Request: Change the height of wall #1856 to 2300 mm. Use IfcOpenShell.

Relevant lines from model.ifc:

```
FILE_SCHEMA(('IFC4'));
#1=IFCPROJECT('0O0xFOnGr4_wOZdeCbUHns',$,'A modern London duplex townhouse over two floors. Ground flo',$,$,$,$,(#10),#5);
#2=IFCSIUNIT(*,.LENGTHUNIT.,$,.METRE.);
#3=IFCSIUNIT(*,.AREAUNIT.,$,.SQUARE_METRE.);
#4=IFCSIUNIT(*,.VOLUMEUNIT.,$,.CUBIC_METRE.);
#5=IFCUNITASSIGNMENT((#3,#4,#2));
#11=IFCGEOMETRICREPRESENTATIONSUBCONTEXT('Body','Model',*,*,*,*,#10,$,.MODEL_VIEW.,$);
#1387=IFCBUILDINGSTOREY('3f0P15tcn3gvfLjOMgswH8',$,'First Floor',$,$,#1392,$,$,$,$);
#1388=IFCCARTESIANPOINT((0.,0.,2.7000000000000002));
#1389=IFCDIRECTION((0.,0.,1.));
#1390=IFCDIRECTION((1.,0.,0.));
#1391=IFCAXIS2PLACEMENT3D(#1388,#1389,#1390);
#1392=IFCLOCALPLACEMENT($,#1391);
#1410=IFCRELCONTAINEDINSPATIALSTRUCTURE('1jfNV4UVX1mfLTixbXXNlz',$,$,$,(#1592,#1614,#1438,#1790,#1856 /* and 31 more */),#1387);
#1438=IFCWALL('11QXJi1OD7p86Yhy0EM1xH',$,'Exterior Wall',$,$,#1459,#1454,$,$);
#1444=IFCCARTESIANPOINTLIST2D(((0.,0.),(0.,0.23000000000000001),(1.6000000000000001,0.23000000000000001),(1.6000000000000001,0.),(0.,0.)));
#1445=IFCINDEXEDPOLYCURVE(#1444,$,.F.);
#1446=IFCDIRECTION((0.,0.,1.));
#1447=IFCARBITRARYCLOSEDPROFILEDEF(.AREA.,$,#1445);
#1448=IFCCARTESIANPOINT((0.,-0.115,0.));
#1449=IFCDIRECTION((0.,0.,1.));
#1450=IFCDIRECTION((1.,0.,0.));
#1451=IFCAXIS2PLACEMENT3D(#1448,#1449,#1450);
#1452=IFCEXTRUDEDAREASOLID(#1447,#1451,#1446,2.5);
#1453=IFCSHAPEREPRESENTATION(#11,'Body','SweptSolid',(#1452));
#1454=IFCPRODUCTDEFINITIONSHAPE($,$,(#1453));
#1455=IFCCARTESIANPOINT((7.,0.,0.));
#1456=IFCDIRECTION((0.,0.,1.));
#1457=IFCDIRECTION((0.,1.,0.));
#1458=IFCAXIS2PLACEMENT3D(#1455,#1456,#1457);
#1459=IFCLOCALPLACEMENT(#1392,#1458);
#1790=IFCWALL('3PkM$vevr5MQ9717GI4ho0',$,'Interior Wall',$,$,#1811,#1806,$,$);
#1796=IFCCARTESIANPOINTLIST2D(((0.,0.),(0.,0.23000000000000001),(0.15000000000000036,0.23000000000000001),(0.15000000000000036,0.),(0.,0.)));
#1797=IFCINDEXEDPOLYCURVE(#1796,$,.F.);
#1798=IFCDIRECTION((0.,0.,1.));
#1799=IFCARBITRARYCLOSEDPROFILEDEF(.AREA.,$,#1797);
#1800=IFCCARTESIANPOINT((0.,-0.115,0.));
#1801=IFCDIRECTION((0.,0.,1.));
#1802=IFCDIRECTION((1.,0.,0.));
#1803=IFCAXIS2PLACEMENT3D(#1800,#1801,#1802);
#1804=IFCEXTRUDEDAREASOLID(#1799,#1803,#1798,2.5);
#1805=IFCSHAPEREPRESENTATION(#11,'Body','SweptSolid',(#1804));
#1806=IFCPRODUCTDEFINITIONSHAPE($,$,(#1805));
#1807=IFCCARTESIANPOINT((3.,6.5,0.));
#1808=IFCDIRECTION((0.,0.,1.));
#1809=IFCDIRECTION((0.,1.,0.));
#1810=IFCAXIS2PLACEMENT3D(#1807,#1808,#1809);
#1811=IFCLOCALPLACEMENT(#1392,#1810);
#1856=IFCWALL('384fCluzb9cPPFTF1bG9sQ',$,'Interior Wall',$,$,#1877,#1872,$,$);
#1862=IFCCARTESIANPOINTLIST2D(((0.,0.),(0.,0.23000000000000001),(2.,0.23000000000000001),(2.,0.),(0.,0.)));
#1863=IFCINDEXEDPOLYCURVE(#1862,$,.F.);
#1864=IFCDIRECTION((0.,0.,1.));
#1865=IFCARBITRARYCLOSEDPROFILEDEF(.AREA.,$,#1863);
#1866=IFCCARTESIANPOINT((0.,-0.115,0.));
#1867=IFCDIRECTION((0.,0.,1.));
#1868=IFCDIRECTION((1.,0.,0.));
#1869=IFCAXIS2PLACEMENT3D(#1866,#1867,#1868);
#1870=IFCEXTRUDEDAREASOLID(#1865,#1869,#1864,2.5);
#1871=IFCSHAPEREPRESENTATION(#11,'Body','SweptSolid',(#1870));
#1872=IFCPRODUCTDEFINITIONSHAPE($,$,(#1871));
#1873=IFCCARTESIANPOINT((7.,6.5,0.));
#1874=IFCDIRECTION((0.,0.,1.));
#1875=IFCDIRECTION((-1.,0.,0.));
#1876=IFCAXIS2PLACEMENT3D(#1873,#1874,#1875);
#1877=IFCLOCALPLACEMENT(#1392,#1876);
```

```python
import ifcopenshell
import ifcopenshell.geom
import ifcopenshell.util.representation
import ifcopenshell.util.shape

model = ifcopenshell.open("model.ifc")
settings = ifcopenshell.geom.settings()


def volume(element):
    """Net volume in cubic metres, openings subtracted."""
    shape = ifcopenshell.geom.create_shape(settings, element)
    return ifcopenshell.util.shape.get_volume(shape.geometry)


wall = model.by_id(1856)
before = volume(wall)

body = ifcopenshell.util.representation.get_representation(wall, "Model", "Body")
solid = body.Items[0]
old_height = solid.Depth
solid.Depth = 2.3
after = volume(wall)

print(f"height {old_height:g} -> {solid.Depth:g}, volume {before:.3f} -> {after:.3f} m3")

model.write("model_v2.ifc")
```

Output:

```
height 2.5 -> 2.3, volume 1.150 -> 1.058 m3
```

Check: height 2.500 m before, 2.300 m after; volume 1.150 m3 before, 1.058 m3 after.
